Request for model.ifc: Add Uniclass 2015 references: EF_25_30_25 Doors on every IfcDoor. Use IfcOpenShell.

First a look at what the model holds.

```python
import ifcopenshell

model = ifcopenshell.open("model.ifc")
print(model.schema)
print("classifications:", [c.Name for c in model.by_type("IfcClassification")])
for ifc_class in ("IfcDoor", "IfcRoof", "IfcStair", "IfcWall", "IfcWindow"):
    print(ifc_class, len(model.by_type(ifc_class)))
```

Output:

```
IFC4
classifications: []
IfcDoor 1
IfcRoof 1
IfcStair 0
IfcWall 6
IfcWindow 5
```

```python
import ifcopenshell
import ifcopenshell.api.classification

model = ifcopenshell.open("model.ifc")

system = ifcopenshell.api.classification.add_classification(model, classification="Uniclass 2015")

codes = {
    "IfcDoor": ("EF_25_30_25", "Doors"),
}
for ifc_class, (code, name) in codes.items():
    products = model.by_type(ifc_class)
    ifcopenshell.api.classification.add_reference(
        model, products=products, classification=system, identification=code, name=name
    )
    print(code, len(products))

model.write("model-out.ifc")
```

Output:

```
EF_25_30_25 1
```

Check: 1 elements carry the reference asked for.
